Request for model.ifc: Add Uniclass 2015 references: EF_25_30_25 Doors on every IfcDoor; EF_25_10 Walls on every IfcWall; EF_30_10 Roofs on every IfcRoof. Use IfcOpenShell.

First a look at what the model holds.

```python
import ifcopenshell

model = ifcopenshell.open("model.ifc")
print(model.schema)
print("classifications:", [c.Name for c in model.by_type("IfcClassification")])
for ifc_class in ("IfcDoor", "IfcRoof", "IfcStair", "IfcWall", "IfcWindow"):
    print(ifc_class, len(model.by_type(ifc_class)))
```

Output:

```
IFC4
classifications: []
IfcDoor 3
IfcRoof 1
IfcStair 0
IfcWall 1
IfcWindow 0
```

```python
import ifcopenshell
import ifcopenshell.api.classification

model = ifcopenshell.open("model.ifc")

system = ifcopenshell.api.classification.add_classification(model, classification="Uniclass 2015")

codes = {
    "IfcDoor": ("EF_25_30_25", "Doors"),
    "IfcWall": ("EF_25_10", "Walls"),
    "IfcRoof": ("EF_30_10", "Roofs"),
}
for ifc_class, (code, name) in codes.items():
    products = model.by_type(ifc_class)
    ifcopenshell.api.classification.add_reference(
        model, products=products, classification=system, identification=code, name=name
    )
    print(code, len(products))

model.write("model_v2.ifc")
```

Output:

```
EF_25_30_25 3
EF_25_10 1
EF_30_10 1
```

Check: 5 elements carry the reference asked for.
